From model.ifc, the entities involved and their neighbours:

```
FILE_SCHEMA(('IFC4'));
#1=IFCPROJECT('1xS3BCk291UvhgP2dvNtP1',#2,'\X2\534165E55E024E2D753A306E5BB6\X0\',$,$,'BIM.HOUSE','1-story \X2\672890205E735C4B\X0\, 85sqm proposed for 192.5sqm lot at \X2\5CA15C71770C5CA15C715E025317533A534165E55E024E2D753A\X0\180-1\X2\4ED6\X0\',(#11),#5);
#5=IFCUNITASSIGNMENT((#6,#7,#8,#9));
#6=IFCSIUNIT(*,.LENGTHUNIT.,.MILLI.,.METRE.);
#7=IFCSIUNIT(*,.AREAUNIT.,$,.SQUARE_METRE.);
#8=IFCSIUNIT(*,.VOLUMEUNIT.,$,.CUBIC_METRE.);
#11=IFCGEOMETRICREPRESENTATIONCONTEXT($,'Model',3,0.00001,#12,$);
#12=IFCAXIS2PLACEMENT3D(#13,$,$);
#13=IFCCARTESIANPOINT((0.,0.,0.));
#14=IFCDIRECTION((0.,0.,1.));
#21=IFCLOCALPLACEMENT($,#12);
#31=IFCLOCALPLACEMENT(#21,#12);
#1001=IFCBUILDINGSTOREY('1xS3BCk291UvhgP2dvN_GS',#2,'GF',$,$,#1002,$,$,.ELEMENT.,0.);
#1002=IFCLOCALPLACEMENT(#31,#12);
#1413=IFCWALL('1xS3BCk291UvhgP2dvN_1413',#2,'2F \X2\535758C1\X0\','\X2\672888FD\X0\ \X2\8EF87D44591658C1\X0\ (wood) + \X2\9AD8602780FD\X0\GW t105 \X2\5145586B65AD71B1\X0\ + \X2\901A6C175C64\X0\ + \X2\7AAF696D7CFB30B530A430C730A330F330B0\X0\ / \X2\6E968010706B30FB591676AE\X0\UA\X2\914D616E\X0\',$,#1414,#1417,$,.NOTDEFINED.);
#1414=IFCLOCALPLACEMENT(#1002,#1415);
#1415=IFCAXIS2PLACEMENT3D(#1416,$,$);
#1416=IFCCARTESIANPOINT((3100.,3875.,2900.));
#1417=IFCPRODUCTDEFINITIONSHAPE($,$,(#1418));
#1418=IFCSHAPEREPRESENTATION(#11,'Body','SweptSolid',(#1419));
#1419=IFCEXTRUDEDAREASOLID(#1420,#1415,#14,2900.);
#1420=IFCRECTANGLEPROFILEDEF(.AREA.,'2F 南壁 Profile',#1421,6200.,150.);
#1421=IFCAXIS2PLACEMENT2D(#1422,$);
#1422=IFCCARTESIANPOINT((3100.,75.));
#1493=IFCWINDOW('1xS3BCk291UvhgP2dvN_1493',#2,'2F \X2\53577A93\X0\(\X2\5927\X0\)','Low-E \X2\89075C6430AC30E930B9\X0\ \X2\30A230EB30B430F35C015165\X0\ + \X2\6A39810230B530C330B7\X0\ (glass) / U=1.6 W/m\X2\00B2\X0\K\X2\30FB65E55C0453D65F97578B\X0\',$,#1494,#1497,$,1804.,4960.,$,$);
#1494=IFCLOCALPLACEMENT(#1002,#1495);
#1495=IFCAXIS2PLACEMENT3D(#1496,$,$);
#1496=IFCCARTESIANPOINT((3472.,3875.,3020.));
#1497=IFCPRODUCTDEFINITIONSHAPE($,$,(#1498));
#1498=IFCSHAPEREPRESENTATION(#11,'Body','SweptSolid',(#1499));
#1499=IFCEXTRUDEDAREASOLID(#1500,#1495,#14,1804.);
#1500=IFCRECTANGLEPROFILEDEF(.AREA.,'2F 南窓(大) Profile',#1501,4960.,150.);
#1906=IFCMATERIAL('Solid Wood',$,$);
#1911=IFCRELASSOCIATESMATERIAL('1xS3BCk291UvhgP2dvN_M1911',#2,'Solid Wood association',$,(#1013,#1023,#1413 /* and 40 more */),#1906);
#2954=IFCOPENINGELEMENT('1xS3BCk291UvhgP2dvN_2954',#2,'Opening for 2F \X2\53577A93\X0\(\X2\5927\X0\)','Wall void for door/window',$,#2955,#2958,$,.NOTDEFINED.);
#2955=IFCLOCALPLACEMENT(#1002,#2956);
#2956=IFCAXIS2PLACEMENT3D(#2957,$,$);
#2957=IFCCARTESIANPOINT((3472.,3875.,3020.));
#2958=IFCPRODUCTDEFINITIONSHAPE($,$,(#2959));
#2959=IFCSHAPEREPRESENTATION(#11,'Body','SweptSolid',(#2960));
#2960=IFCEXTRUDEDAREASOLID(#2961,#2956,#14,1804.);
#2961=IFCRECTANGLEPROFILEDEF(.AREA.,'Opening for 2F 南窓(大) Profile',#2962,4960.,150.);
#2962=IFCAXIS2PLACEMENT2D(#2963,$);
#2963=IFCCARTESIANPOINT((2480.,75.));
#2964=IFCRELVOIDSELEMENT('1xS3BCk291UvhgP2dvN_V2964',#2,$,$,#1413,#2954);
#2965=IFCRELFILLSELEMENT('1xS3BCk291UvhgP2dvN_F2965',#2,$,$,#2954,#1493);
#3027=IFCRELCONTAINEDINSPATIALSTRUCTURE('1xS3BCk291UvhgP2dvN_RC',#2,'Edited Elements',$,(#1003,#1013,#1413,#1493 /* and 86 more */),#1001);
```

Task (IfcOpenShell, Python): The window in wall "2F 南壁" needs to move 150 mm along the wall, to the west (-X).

```python
import ifcopenshell
import ifcopenshell.api.geometry
import ifcopenshell.util.placement
import ifcopenshell.util.unit

model = ifcopenshell.open("model.ifc")
unit_scale = ifcopenshell.util.unit.calculate_unit_scale(model)

window = model.by_guid("1xS3BCk291UvhgP2dvN_1493")
opening = window.FillsVoids[0].RelatingOpeningElement
wall = opening.VoidsElements[0].RelatingBuildingElement

wall_matrix = ifcopenshell.util.placement.get_local_placement(wall.ObjectPlacement)
shift = wall_matrix[:3, 0] * -0.15 / unit_scale
before = ifcopenshell.util.placement.get_local_placement(window.ObjectPlacement)[:3, 3].copy()

# The window is not placed relative to its opening, so move both.
for product in (opening, window):
    matrix = ifcopenshell.util.placement.get_local_placement(product.ObjectPlacement)
    matrix[:3, 3] += shift
    ifcopenshell.api.geometry.edit_object_placement(model, product=product, matrix=matrix, is_si=False)

after = ifcopenshell.util.placement.get_local_placement(window.ObjectPlacement)[:3, 3]
print("window moved by", (after - before).round(3) + 0.0)

model.write("model_updated.ifc")
```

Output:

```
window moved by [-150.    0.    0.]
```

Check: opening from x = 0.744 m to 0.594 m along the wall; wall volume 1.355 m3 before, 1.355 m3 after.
